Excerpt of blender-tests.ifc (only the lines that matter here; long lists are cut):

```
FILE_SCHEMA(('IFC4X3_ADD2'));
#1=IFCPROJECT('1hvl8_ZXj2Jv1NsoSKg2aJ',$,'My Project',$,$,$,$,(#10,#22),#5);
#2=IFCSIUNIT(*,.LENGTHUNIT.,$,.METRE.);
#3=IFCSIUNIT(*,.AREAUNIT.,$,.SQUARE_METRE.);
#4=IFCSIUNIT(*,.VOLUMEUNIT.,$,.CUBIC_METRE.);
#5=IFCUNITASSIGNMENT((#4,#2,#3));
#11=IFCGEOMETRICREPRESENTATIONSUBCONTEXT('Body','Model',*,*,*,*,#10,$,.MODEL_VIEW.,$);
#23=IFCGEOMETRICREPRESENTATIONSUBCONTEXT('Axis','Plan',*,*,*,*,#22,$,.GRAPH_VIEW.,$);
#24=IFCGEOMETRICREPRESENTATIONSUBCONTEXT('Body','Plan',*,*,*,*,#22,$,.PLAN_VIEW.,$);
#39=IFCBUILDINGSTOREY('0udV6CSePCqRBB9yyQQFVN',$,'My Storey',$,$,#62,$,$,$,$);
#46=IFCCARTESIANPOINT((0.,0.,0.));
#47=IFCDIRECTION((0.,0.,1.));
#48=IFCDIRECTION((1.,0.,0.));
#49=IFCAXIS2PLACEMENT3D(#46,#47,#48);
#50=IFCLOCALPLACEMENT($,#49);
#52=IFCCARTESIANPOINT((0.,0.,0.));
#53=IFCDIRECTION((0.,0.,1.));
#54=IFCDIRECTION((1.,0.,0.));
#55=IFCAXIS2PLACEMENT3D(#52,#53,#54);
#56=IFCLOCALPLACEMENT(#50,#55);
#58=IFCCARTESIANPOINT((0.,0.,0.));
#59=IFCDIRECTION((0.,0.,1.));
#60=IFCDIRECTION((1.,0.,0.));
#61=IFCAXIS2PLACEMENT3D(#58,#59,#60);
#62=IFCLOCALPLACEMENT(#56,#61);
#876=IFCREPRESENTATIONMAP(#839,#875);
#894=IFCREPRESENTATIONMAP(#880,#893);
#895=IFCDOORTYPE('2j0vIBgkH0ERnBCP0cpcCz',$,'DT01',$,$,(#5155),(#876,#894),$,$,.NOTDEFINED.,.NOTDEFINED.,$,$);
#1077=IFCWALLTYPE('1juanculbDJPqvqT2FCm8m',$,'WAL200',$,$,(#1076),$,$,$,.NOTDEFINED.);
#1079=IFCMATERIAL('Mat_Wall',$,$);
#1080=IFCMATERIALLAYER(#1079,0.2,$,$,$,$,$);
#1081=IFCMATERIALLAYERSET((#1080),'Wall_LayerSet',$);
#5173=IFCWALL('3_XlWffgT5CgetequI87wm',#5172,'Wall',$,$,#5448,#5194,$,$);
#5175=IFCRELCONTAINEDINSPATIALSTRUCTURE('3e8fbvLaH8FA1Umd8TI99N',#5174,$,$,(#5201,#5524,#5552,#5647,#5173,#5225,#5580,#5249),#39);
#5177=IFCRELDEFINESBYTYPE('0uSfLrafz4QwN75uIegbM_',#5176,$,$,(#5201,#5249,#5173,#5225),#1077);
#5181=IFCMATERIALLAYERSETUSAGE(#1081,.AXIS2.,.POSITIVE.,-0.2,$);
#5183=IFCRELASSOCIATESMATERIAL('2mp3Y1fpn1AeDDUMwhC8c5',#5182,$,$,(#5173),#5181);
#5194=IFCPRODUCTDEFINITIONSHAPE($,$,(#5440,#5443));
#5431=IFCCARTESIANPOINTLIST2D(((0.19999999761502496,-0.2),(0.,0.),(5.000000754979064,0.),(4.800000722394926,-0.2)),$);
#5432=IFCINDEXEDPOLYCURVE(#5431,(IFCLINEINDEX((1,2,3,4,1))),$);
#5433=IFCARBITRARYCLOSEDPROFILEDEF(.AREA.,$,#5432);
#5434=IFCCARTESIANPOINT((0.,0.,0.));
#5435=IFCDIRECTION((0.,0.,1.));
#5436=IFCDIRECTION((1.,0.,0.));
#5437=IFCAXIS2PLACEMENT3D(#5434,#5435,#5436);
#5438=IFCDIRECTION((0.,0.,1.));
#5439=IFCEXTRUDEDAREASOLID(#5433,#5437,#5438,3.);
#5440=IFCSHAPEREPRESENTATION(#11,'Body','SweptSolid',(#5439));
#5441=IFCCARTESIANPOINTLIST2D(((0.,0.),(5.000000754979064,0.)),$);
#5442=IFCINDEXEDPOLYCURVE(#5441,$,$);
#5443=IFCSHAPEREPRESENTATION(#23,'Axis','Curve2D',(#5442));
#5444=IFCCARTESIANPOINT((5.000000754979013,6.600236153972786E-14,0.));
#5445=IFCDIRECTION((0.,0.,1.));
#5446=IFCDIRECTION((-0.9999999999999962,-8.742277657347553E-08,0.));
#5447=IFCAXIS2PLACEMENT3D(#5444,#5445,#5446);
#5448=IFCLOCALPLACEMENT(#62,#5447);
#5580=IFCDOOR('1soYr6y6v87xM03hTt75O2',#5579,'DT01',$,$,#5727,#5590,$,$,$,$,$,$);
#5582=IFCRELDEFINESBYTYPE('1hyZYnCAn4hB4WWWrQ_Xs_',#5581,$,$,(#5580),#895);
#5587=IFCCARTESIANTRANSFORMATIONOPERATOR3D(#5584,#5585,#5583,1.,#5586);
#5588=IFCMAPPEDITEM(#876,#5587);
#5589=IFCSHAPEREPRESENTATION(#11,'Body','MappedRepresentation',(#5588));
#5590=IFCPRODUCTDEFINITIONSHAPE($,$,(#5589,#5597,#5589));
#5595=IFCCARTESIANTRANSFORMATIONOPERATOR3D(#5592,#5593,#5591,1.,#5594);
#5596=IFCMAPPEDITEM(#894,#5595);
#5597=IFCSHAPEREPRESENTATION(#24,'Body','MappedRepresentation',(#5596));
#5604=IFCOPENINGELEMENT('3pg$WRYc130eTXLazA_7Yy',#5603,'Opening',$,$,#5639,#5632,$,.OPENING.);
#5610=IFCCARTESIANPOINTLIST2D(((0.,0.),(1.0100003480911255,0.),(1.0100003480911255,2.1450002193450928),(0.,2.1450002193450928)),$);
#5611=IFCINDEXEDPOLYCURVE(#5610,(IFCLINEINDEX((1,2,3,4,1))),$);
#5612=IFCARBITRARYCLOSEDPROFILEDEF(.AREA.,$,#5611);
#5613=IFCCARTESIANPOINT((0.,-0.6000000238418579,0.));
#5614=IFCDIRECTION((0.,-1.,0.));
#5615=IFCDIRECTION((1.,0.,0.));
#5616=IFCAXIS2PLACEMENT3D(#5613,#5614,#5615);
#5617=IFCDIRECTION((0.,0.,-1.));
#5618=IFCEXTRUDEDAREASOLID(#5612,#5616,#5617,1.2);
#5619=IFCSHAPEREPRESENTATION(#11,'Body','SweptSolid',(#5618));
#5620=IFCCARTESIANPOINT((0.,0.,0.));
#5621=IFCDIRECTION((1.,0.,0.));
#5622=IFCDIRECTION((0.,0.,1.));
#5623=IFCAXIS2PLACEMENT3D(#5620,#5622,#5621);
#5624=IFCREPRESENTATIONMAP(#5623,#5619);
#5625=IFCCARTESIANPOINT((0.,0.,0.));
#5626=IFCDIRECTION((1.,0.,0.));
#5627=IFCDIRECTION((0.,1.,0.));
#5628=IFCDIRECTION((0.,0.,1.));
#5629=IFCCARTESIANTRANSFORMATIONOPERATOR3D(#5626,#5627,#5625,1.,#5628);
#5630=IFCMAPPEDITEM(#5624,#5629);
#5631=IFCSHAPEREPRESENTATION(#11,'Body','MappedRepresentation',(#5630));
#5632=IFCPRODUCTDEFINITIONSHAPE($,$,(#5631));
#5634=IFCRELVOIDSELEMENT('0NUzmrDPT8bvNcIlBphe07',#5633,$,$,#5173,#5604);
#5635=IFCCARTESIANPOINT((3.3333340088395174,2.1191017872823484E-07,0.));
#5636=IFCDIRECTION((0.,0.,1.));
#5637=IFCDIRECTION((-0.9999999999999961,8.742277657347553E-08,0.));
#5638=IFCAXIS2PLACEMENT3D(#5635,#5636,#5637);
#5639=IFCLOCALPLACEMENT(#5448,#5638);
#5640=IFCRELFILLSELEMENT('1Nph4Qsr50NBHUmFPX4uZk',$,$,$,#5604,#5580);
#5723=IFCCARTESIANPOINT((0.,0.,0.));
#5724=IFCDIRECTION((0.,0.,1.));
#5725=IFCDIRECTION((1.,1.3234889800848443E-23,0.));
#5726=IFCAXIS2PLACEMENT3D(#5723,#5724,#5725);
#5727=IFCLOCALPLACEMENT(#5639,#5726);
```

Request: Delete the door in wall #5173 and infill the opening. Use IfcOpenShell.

```python
import ifcopenshell
import ifcopenshell.api.feature
import ifcopenshell.api.root
import ifcopenshell.geom
import ifcopenshell.util.shape

model = ifcopenshell.open("blender-tests.ifc")
settings = ifcopenshell.geom.settings()


def volume(element):
    """Net volume in cubic metres, openings subtracted."""
    shape = ifcopenshell.geom.create_shape(settings, element)
    return ifcopenshell.util.shape.get_volume(shape.geometry)


door = model.by_id(5580)
opening = door.FillsVoids[0].RelatingOpeningElement
wall = opening.VoidsElements[0].RelatingBuildingElement
before = volume(wall)

ifcopenshell.api.root.remove_product(model, product=door)
ifcopenshell.api.feature.remove_feature(model, feature=opening)

after = volume(wall)

print(f"wall volume {before:.3f} -> {after:.3f} m3")

model.write("blender-tests_rev.ifc")
```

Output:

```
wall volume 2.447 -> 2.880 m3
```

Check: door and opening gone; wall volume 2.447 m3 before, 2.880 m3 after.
